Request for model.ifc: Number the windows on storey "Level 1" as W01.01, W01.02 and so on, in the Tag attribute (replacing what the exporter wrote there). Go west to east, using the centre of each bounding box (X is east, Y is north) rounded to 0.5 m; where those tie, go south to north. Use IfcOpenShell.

First a look at what the model holds.

```python
import ifcopenshell
import ifcopenshell.util.element
import ifcopenshell.util.placement

model = ifcopenshell.open("model.ifc")
print(model.schema)
storey = next(s for s in model.by_type("IfcBuildingStorey") if s.Name == "Level 1")
windows = [e for e in ifcopenshell.util.element.get_decomposition(storey) if e.is_a("IfcWindow")]
for e in sorted(windows, key=lambda e: e.id()):
    origin = ifcopenshell.util.placement.get_local_placement(e.ObjectPlacement)[:3, 3]
    print(e.id(), e.Tag, e.Name, origin.round(2) + 0.0, sep=" | ")
```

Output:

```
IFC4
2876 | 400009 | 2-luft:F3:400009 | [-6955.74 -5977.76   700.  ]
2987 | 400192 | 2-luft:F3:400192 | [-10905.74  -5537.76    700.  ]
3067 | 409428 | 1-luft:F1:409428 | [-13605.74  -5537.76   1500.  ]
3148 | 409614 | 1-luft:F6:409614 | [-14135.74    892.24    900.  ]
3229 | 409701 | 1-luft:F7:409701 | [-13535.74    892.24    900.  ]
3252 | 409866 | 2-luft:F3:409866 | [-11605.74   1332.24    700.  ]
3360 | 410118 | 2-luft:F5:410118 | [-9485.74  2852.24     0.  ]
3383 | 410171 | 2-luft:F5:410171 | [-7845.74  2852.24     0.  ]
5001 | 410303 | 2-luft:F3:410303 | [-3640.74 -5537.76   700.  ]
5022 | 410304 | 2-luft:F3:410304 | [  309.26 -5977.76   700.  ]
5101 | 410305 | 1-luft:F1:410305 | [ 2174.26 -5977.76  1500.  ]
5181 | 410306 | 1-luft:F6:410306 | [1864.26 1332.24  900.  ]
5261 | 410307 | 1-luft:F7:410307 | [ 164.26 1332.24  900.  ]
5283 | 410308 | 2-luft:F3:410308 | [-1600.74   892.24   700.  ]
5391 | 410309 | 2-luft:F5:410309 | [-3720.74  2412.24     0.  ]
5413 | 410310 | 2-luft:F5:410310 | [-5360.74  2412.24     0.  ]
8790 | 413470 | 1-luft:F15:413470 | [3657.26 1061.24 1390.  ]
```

```python
import ifcopenshell
import ifcopenshell.geom
import ifcopenshell.util.element
import ifcopenshell.util.shape

model = ifcopenshell.open("model.ifc")
settings = ifcopenshell.geom.settings()
settings.set("use-world-coords", True)


def centre(element):
    shape = ifcopenshell.geom.create_shape(settings, element)
    return ifcopenshell.util.shape.get_bbox_centroid(shape.geometry)


storey = next(s for s in model.by_type("IfcBuildingStorey") if s.Name == "Level 1")
windows = [e for e in ifcopenshell.util.element.get_decomposition(storey) if e.is_a("IfcWindow")]

# Insertion points can sit at a corner or the storey origin, so sort by the geometry (in metres).
centres = {e: centre(e) for e in windows}
windows.sort(key=lambda e: (round(centres[e][0] / 0.5), centres[e][1]))

for i, e in enumerate(windows, start=1):
    number = f"W01.{i:02d}"
    e.Tag = number
    print(e.id(), number)

model.write("model_edited.ifc")
```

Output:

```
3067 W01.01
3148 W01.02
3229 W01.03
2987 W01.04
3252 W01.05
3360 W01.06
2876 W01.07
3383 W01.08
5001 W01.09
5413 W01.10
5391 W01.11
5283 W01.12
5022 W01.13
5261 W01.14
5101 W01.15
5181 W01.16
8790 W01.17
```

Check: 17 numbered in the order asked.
